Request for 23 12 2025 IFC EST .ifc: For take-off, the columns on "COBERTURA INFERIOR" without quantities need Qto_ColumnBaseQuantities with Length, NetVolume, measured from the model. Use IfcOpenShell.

First a look at what the model holds.

```python
import ifcopenshell
import ifcopenshell.util.element
import ifcopenshell.util.unit

model = ifcopenshell.open("23 12 2025 IFC EST .ifc")
print(model.schema)
for unit_type in ("LENGTHUNIT", "AREAUNIT", "VOLUMEUNIT"):
    print(unit_type, ifcopenshell.util.unit.calculate_unit_scale(model, unit_type))
storey = next(s for s in model.by_type("IfcBuildingStorey") if s.Name == "COBERTURA INFERIOR")
columns = [e for e in ifcopenshell.util.element.get_decomposition(storey) if e.is_a("IfcColumn")]
for e in sorted(columns, key=lambda e: e.id()):
    print(e.id(), e.is_a(), e.Name, list(ifcopenshell.util.element.get_psets(e, qtos_only=True)), sep=" | ")
```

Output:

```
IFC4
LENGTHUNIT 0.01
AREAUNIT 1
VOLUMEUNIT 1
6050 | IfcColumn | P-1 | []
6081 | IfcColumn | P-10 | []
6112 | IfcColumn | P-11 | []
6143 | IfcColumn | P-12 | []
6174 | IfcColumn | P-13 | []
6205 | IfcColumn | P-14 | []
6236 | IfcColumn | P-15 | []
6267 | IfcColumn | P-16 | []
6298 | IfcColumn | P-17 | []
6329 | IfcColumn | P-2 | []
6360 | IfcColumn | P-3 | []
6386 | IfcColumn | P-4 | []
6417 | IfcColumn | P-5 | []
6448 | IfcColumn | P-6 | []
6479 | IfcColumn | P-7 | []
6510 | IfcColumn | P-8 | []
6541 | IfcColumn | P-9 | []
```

```python
import ifcopenshell
import ifcopenshell.api.pset
import ifcopenshell.geom
import ifcopenshell.util.element
import ifcopenshell.util.shape
import ifcopenshell.util.unit

model = ifcopenshell.open("23 12 2025 IFC EST .ifc")
unit_scale = ifcopenshell.util.unit.calculate_unit_scale(model)
volume_scale = ifcopenshell.util.unit.calculate_unit_scale(model, "VOLUMEUNIT")
settings = ifcopenshell.geom.settings()

storey = next(s for s in model.by_type("IfcBuildingStorey") if s.Name == "COBERTURA INFERIOR")
columns = [e for e in ifcopenshell.util.element.get_decomposition(storey) if e.is_a("IfcColumn")]

for e in sorted(columns, key=lambda e: e.id()):
    if ifcopenshell.util.element.get_psets(e, qtos_only=True, should_inherit=False):
        continue
    # Geometry comes back in metres, in the element's own axes.
    shape = ifcopenshell.geom.create_shape(settings, e)
    values = {
        "Length": ifcopenshell.util.shape.get_z(shape.geometry) / unit_scale,
        "NetVolume": ifcopenshell.util.shape.get_volume(shape.geometry) / volume_scale,
    }
    qto = ifcopenshell.api.pset.add_qto(model, product=e, name="Qto_ColumnBaseQuantities")
    ifcopenshell.api.pset.edit_qto(model, qto=qto, properties=values)
    print(e.id(), {k: round(v, 3) for k, v in values.items()})

model.write("23 12 2025 IFC EST _edited.ifc")
```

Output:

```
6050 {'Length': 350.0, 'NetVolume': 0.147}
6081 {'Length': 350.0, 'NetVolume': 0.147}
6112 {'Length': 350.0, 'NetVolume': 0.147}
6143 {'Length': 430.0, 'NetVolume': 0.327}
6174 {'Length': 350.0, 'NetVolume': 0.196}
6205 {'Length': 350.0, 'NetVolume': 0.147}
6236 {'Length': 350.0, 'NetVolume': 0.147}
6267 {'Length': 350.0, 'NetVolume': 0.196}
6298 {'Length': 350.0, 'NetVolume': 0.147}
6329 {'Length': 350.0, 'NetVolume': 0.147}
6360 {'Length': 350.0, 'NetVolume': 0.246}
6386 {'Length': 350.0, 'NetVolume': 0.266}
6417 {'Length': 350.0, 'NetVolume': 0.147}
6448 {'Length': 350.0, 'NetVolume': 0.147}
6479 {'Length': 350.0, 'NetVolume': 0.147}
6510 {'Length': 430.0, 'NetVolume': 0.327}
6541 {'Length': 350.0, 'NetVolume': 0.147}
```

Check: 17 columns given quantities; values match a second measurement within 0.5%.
